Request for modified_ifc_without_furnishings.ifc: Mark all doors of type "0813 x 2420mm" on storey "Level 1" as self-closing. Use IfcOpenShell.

First a look at what the model holds.

```python
import ifcopenshell
import ifcopenshell.util.element

model = ifcopenshell.open("modified_ifc_without_furnishings.ifc")
print(model.schema)
storey = next(s for s in model.by_type("IfcBuildingStorey") if s.Name == "Level 1")
doors = [e for e in ifcopenshell.util.element.get_decomposition(storey) if e.is_a("IfcDoor")]
seen = {}
for e in doors:
    element_type = ifcopenshell.util.element.get_type(e)
    key = (element_type.Name if element_type != e and element_type else None, ifcopenshell.util.element.get_pset(e, "Pset_DoorCommon", "SelfClosing"))
    seen[key] = seen.get(key, 0) + 1
for (name, value), count in sorted(seen.items(), key=str):
    print(count, "x", name, "|", value)
```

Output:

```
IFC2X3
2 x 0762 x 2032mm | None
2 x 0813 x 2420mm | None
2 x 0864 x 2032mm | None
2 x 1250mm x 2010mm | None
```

```python
import ifcopenshell
import ifcopenshell.api.pset
import ifcopenshell.util.element

model = ifcopenshell.open("modified_ifc_without_furnishings.ifc")

storey = next(s for s in model.by_type("IfcBuildingStorey") if s.Name == "Level 1")
doors = [e for e in ifcopenshell.util.element.get_decomposition(storey) if e.is_a("IfcDoor")]

count = 0
for e in doors:
    element_type = ifcopenshell.util.element.get_type(e)
    if element_type in (None, e) or element_type.Name != "0813 x 2420mm":
        continue
    # add_pset returns the element's existing set when there is one.
    pset = ifcopenshell.api.pset.add_pset(model, product=e, name="Pset_DoorCommon")
    ifcopenshell.api.pset.edit_pset(model, pset=pset, properties={"SelfClosing": True})
    count += 1

print(count, "doors updated")

model.write("modified_ifc_without_furnishings_edited.ifc")
```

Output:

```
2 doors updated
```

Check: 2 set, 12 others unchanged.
